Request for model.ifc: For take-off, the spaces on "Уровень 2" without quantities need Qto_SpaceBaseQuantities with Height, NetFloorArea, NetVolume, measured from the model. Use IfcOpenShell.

First a look at what the model holds.

```python
import ifcopenshell
import ifcopenshell.util.element
import ifcopenshell.util.unit

model = ifcopenshell.open("model.ifc")
print(model.schema)
for unit_type in ("LENGTHUNIT", "AREAUNIT", "VOLUMEUNIT"):
    print(unit_type, ifcopenshell.util.unit.calculate_unit_scale(model, unit_type))
storey = next(s for s in model.by_type("IfcBuildingStorey") if s.Name == "Уровень 2")
spaces = [e for e in ifcopenshell.util.element.get_decomposition(storey) if e.is_a("IfcSpace")]
for e in sorted(spaces, key=lambda e: e.id()):
    print(e.id(), e.is_a(), e.Name, list(ifcopenshell.util.element.get_psets(e, qtos_only=True)), sep=" | ")
```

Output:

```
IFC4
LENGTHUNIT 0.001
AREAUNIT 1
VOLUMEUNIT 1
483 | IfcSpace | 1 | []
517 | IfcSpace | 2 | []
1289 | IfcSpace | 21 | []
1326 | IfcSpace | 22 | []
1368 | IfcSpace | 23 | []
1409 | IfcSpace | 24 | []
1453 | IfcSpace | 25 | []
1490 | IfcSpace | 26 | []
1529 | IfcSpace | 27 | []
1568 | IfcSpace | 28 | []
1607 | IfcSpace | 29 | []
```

```python
import ifcopenshell
import ifcopenshell.api.pset
import ifcopenshell.geom
import ifcopenshell.util.element
import ifcopenshell.util.shape
import ifcopenshell.util.unit

model = ifcopenshell.open("model.ifc")
unit_scale = ifcopenshell.util.unit.calculate_unit_scale(model)
area_scale = ifcopenshell.util.unit.calculate_unit_scale(model, "AREAUNIT")
volume_scale = ifcopenshell.util.unit.calculate_unit_scale(model, "VOLUMEUNIT")
settings = ifcopenshell.geom.settings()

storey = next(s for s in model.by_type("IfcBuildingStorey") if s.Name == "Уровень 2")
spaces = [e for e in ifcopenshell.util.element.get_decomposition(storey) if e.is_a("IfcSpace")]

for e in sorted(spaces, key=lambda e: e.id()):
    if ifcopenshell.util.element.get_psets(e, qtos_only=True, should_inherit=False):
        continue
    # Geometry comes back in metres, in the element's own axes.
    shape = ifcopenshell.geom.create_shape(settings, e)
    values = {
        "Height": ifcopenshell.util.shape.get_z(shape.geometry) / unit_scale,
        "NetFloorArea": ifcopenshell.util.shape.get_footprint_area(shape.geometry) / area_scale,
        "NetVolume": ifcopenshell.util.shape.get_volume(shape.geometry) / volume_scale,
    }
    qto = ifcopenshell.api.pset.add_qto(model, product=e, name="Qto_SpaceBaseQuantities")
    ifcopenshell.api.pset.edit_qto(model, qto=qto, properties=values)
    print(e.id(), {k: round(v, 3) for k, v in values.items()})

model.write("model_v2.ifc")
```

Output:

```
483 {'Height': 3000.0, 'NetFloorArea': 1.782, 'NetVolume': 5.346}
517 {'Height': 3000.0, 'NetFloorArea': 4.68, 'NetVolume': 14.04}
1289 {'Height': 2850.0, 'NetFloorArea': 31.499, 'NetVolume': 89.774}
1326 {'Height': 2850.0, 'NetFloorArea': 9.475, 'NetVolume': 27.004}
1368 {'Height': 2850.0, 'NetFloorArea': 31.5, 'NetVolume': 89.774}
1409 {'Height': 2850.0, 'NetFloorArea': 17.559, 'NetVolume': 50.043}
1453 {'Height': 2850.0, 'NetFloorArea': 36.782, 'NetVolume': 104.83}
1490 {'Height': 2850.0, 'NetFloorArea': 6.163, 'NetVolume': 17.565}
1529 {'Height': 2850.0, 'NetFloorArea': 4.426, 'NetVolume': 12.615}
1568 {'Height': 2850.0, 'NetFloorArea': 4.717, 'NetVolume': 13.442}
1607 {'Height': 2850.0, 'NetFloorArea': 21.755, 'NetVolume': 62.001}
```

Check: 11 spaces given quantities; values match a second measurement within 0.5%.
